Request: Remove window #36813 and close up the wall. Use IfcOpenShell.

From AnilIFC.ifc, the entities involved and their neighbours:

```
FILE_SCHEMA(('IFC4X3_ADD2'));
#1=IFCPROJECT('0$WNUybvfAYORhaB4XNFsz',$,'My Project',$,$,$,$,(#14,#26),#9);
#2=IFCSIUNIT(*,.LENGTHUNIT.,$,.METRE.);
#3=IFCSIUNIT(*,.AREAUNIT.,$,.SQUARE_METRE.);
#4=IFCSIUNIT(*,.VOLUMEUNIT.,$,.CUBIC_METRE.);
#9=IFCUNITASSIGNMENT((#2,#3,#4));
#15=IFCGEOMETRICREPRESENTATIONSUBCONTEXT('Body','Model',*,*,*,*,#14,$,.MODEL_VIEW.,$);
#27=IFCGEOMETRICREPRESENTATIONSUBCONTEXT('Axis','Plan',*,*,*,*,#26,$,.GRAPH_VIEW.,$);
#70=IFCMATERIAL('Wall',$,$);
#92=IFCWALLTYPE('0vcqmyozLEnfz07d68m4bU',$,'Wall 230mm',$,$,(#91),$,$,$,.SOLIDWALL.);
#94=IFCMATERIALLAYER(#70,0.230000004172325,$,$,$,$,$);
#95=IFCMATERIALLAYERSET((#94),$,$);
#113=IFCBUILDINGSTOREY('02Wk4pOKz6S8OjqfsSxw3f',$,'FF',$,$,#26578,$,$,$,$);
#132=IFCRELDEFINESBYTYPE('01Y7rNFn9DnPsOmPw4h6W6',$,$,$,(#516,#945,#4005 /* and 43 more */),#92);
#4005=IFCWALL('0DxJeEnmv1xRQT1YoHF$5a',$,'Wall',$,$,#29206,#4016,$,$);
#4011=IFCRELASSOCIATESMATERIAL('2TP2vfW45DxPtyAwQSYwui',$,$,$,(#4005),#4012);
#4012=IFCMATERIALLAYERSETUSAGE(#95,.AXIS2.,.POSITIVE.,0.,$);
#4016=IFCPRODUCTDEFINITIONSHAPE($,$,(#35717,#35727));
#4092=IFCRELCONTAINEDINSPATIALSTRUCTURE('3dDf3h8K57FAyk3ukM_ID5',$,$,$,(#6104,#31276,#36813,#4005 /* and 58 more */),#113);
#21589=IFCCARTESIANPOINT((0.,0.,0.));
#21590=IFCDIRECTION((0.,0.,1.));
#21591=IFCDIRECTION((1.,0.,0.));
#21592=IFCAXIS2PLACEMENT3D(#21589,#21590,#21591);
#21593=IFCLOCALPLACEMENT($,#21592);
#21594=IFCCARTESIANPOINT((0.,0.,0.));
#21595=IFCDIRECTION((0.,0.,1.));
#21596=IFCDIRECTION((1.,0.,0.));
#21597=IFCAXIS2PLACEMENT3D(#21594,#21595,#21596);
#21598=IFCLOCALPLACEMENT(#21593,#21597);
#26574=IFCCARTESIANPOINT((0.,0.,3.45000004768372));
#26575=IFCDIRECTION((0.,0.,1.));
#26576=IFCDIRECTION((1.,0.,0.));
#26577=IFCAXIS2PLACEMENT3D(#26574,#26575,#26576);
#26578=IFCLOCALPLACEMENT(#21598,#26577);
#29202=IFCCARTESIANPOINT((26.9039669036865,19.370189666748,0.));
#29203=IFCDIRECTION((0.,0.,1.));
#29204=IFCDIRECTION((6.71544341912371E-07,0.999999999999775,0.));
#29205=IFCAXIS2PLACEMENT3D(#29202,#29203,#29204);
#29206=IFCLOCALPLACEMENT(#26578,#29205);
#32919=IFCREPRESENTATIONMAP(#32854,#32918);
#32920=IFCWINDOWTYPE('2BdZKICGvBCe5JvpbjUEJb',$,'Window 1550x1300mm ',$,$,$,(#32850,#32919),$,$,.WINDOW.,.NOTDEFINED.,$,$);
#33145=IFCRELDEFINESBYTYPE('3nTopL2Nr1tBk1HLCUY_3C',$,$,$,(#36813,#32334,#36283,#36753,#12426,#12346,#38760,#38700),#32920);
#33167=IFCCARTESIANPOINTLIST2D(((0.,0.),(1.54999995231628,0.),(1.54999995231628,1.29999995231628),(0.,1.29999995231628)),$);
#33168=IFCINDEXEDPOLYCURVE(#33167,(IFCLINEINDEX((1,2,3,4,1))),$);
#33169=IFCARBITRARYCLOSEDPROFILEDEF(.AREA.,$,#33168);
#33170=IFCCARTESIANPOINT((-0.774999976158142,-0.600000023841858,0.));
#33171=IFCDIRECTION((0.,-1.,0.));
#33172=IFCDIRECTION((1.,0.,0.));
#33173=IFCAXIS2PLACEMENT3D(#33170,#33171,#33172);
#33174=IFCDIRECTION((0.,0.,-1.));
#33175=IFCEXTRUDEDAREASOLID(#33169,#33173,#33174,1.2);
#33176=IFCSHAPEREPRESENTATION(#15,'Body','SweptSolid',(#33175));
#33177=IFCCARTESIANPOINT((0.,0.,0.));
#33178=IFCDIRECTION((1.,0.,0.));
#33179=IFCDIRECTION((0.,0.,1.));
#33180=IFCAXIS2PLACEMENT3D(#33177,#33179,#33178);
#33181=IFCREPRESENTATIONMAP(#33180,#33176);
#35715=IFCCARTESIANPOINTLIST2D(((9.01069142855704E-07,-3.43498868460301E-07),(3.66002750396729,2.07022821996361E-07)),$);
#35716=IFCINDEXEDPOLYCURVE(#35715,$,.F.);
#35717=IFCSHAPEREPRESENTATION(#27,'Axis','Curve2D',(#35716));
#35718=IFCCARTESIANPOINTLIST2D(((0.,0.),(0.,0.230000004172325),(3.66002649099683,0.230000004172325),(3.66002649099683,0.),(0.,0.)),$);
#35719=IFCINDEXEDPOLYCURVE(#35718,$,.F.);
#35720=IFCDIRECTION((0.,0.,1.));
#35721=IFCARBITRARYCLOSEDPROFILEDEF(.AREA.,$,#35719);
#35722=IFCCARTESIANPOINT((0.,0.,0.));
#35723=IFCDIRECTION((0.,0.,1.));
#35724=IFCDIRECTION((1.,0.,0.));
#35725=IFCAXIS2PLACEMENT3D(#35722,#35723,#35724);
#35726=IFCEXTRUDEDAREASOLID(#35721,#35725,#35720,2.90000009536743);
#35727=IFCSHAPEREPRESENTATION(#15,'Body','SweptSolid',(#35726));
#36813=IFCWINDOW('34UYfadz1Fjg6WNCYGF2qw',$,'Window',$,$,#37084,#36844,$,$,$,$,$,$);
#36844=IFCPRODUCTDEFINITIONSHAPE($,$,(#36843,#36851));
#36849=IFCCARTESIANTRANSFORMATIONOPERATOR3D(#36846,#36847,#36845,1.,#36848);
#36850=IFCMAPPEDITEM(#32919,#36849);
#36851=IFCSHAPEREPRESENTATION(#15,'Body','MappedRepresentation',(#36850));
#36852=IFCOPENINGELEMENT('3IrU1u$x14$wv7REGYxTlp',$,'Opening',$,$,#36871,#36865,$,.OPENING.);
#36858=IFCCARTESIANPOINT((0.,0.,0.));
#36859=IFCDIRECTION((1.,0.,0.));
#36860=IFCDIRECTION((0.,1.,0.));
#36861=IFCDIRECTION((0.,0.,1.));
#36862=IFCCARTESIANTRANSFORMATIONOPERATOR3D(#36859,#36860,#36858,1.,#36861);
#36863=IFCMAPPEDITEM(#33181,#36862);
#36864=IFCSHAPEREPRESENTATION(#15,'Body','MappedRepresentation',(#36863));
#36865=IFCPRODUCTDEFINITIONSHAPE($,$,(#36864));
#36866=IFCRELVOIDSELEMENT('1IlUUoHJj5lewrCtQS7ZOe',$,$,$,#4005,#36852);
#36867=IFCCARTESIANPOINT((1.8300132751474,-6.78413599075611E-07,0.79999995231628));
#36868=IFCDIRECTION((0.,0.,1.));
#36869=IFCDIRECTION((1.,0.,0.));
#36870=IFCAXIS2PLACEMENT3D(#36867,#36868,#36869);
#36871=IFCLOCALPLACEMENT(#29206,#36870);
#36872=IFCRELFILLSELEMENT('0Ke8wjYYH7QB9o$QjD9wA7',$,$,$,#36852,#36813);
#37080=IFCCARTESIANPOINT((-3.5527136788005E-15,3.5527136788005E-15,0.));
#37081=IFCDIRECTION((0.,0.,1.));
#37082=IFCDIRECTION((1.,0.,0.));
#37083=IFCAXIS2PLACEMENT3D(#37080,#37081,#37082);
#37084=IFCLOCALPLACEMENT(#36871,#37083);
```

```python
import ifcopenshell
import ifcopenshell.api.feature
import ifcopenshell.api.root
import ifcopenshell.geom
import ifcopenshell.util.shape

model = ifcopenshell.open("AnilIFC.ifc")
settings = ifcopenshell.geom.settings()


def volume(element):
    """Net volume in cubic metres, openings subtracted."""
    shape = ifcopenshell.geom.create_shape(settings, element)
    return ifcopenshell.util.shape.get_volume(shape.geometry)


window = model.by_id(36813)
opening = window.FillsVoids[0].RelatingOpeningElement
wall = opening.VoidsElements[0].RelatingBuildingElement
before = volume(wall)

ifcopenshell.api.root.remove_product(model, product=window)
ifcopenshell.api.feature.remove_feature(model, feature=opening)

after = volume(wall)

print(f"wall volume {before:.3f} -> {after:.3f} m3")

model.write("AnilIFC_v2.ifc")
```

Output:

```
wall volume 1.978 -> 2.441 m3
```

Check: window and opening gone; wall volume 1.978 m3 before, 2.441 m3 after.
